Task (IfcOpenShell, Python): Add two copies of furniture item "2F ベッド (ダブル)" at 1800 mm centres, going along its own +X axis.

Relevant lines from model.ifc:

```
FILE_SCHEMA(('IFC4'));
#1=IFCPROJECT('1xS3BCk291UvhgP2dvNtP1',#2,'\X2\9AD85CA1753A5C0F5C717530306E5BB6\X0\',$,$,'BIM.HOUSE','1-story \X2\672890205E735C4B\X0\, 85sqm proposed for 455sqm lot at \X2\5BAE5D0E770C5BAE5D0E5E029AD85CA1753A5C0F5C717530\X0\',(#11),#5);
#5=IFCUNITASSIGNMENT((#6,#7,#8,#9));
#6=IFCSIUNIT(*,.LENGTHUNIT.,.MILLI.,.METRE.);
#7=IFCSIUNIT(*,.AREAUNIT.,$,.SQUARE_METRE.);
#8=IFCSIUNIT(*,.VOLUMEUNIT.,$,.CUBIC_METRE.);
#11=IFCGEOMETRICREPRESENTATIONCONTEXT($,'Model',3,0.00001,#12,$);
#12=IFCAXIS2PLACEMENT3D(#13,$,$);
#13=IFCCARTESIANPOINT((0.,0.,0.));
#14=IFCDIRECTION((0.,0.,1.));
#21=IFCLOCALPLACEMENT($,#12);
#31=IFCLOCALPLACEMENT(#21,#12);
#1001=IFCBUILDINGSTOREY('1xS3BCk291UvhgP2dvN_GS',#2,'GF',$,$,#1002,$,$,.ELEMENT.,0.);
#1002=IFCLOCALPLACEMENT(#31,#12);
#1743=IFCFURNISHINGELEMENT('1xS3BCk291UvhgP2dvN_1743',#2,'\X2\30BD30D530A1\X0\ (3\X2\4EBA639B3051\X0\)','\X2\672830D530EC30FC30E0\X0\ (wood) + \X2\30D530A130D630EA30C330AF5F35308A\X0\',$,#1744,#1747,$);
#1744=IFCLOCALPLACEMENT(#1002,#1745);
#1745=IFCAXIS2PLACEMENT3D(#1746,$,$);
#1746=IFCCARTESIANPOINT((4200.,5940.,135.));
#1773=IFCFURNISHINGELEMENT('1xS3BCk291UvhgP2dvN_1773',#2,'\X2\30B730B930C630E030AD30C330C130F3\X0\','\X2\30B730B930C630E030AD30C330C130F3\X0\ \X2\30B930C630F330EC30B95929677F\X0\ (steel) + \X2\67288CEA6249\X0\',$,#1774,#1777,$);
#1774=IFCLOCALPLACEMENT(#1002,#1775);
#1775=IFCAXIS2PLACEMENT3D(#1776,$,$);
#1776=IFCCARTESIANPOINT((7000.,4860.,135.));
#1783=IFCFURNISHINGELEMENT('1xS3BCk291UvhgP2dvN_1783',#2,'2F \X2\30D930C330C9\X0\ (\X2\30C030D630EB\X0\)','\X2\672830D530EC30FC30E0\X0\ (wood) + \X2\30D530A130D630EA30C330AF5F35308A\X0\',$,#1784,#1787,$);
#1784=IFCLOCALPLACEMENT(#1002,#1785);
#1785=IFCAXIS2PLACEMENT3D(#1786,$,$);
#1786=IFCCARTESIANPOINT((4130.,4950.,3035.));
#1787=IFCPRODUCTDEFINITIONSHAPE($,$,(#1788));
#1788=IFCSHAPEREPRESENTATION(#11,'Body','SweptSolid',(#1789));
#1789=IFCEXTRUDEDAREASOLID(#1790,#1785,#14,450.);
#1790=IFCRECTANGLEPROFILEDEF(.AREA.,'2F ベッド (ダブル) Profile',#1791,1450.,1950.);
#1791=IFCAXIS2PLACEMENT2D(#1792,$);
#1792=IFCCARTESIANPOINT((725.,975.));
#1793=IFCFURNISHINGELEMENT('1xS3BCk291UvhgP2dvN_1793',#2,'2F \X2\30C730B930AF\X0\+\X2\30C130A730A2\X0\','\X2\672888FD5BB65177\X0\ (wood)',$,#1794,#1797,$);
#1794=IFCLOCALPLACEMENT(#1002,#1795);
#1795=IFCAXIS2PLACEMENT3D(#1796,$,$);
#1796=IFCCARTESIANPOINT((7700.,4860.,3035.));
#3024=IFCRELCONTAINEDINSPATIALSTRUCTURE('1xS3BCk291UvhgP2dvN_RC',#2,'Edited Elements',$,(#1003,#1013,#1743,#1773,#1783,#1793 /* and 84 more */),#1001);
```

```python
import ifcopenshell
import ifcopenshell.api.geometry
import ifcopenshell.api.root
import ifcopenshell.util.element
import ifcopenshell.util.placement

model = ifcopenshell.open("model.ifc")


def reuse_history(source, copy):
    """copy_class also copies each property set's owner history, people and application; keep the originals."""
    for rel in copy.IsDefinedBy:
        if rel.is_a("IfcRelDefinesByProperties") and (history := rel.RelatingPropertyDefinition.OwnerHistory):
            rel.RelatingPropertyDefinition.OwnerHistory = source.OwnerHistory
            ifcopenshell.util.element.remove_deep2(model, history)


source = model.by_guid("1xS3BCk291UvhgP2dvN_1783")
base = ifcopenshell.util.placement.get_local_placement(source.ObjectPlacement)
step = base[:3, 0] * 1800.0

for i in range(1, 3):
    copy = ifcopenshell.api.root.copy_class(model, product=source)
    copy.Representation = ifcopenshell.util.element.copy_deep(
        model, source.Representation, exclude=["IfcGeometricRepresentationContext", "IfcRepresentationMap"]
    )
    reuse_history(source, copy)
    matrix = base.copy()
    matrix[:3, 3] += i * step
    print("added at", matrix[:3, 3].round(3) + 0.0)
    ifcopenshell.api.geometry.edit_object_placement(model, product=copy, matrix=matrix, is_si=False)

model.write("model_edited.ifc")
```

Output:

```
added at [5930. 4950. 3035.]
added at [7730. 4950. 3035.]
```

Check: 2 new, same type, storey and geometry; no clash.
